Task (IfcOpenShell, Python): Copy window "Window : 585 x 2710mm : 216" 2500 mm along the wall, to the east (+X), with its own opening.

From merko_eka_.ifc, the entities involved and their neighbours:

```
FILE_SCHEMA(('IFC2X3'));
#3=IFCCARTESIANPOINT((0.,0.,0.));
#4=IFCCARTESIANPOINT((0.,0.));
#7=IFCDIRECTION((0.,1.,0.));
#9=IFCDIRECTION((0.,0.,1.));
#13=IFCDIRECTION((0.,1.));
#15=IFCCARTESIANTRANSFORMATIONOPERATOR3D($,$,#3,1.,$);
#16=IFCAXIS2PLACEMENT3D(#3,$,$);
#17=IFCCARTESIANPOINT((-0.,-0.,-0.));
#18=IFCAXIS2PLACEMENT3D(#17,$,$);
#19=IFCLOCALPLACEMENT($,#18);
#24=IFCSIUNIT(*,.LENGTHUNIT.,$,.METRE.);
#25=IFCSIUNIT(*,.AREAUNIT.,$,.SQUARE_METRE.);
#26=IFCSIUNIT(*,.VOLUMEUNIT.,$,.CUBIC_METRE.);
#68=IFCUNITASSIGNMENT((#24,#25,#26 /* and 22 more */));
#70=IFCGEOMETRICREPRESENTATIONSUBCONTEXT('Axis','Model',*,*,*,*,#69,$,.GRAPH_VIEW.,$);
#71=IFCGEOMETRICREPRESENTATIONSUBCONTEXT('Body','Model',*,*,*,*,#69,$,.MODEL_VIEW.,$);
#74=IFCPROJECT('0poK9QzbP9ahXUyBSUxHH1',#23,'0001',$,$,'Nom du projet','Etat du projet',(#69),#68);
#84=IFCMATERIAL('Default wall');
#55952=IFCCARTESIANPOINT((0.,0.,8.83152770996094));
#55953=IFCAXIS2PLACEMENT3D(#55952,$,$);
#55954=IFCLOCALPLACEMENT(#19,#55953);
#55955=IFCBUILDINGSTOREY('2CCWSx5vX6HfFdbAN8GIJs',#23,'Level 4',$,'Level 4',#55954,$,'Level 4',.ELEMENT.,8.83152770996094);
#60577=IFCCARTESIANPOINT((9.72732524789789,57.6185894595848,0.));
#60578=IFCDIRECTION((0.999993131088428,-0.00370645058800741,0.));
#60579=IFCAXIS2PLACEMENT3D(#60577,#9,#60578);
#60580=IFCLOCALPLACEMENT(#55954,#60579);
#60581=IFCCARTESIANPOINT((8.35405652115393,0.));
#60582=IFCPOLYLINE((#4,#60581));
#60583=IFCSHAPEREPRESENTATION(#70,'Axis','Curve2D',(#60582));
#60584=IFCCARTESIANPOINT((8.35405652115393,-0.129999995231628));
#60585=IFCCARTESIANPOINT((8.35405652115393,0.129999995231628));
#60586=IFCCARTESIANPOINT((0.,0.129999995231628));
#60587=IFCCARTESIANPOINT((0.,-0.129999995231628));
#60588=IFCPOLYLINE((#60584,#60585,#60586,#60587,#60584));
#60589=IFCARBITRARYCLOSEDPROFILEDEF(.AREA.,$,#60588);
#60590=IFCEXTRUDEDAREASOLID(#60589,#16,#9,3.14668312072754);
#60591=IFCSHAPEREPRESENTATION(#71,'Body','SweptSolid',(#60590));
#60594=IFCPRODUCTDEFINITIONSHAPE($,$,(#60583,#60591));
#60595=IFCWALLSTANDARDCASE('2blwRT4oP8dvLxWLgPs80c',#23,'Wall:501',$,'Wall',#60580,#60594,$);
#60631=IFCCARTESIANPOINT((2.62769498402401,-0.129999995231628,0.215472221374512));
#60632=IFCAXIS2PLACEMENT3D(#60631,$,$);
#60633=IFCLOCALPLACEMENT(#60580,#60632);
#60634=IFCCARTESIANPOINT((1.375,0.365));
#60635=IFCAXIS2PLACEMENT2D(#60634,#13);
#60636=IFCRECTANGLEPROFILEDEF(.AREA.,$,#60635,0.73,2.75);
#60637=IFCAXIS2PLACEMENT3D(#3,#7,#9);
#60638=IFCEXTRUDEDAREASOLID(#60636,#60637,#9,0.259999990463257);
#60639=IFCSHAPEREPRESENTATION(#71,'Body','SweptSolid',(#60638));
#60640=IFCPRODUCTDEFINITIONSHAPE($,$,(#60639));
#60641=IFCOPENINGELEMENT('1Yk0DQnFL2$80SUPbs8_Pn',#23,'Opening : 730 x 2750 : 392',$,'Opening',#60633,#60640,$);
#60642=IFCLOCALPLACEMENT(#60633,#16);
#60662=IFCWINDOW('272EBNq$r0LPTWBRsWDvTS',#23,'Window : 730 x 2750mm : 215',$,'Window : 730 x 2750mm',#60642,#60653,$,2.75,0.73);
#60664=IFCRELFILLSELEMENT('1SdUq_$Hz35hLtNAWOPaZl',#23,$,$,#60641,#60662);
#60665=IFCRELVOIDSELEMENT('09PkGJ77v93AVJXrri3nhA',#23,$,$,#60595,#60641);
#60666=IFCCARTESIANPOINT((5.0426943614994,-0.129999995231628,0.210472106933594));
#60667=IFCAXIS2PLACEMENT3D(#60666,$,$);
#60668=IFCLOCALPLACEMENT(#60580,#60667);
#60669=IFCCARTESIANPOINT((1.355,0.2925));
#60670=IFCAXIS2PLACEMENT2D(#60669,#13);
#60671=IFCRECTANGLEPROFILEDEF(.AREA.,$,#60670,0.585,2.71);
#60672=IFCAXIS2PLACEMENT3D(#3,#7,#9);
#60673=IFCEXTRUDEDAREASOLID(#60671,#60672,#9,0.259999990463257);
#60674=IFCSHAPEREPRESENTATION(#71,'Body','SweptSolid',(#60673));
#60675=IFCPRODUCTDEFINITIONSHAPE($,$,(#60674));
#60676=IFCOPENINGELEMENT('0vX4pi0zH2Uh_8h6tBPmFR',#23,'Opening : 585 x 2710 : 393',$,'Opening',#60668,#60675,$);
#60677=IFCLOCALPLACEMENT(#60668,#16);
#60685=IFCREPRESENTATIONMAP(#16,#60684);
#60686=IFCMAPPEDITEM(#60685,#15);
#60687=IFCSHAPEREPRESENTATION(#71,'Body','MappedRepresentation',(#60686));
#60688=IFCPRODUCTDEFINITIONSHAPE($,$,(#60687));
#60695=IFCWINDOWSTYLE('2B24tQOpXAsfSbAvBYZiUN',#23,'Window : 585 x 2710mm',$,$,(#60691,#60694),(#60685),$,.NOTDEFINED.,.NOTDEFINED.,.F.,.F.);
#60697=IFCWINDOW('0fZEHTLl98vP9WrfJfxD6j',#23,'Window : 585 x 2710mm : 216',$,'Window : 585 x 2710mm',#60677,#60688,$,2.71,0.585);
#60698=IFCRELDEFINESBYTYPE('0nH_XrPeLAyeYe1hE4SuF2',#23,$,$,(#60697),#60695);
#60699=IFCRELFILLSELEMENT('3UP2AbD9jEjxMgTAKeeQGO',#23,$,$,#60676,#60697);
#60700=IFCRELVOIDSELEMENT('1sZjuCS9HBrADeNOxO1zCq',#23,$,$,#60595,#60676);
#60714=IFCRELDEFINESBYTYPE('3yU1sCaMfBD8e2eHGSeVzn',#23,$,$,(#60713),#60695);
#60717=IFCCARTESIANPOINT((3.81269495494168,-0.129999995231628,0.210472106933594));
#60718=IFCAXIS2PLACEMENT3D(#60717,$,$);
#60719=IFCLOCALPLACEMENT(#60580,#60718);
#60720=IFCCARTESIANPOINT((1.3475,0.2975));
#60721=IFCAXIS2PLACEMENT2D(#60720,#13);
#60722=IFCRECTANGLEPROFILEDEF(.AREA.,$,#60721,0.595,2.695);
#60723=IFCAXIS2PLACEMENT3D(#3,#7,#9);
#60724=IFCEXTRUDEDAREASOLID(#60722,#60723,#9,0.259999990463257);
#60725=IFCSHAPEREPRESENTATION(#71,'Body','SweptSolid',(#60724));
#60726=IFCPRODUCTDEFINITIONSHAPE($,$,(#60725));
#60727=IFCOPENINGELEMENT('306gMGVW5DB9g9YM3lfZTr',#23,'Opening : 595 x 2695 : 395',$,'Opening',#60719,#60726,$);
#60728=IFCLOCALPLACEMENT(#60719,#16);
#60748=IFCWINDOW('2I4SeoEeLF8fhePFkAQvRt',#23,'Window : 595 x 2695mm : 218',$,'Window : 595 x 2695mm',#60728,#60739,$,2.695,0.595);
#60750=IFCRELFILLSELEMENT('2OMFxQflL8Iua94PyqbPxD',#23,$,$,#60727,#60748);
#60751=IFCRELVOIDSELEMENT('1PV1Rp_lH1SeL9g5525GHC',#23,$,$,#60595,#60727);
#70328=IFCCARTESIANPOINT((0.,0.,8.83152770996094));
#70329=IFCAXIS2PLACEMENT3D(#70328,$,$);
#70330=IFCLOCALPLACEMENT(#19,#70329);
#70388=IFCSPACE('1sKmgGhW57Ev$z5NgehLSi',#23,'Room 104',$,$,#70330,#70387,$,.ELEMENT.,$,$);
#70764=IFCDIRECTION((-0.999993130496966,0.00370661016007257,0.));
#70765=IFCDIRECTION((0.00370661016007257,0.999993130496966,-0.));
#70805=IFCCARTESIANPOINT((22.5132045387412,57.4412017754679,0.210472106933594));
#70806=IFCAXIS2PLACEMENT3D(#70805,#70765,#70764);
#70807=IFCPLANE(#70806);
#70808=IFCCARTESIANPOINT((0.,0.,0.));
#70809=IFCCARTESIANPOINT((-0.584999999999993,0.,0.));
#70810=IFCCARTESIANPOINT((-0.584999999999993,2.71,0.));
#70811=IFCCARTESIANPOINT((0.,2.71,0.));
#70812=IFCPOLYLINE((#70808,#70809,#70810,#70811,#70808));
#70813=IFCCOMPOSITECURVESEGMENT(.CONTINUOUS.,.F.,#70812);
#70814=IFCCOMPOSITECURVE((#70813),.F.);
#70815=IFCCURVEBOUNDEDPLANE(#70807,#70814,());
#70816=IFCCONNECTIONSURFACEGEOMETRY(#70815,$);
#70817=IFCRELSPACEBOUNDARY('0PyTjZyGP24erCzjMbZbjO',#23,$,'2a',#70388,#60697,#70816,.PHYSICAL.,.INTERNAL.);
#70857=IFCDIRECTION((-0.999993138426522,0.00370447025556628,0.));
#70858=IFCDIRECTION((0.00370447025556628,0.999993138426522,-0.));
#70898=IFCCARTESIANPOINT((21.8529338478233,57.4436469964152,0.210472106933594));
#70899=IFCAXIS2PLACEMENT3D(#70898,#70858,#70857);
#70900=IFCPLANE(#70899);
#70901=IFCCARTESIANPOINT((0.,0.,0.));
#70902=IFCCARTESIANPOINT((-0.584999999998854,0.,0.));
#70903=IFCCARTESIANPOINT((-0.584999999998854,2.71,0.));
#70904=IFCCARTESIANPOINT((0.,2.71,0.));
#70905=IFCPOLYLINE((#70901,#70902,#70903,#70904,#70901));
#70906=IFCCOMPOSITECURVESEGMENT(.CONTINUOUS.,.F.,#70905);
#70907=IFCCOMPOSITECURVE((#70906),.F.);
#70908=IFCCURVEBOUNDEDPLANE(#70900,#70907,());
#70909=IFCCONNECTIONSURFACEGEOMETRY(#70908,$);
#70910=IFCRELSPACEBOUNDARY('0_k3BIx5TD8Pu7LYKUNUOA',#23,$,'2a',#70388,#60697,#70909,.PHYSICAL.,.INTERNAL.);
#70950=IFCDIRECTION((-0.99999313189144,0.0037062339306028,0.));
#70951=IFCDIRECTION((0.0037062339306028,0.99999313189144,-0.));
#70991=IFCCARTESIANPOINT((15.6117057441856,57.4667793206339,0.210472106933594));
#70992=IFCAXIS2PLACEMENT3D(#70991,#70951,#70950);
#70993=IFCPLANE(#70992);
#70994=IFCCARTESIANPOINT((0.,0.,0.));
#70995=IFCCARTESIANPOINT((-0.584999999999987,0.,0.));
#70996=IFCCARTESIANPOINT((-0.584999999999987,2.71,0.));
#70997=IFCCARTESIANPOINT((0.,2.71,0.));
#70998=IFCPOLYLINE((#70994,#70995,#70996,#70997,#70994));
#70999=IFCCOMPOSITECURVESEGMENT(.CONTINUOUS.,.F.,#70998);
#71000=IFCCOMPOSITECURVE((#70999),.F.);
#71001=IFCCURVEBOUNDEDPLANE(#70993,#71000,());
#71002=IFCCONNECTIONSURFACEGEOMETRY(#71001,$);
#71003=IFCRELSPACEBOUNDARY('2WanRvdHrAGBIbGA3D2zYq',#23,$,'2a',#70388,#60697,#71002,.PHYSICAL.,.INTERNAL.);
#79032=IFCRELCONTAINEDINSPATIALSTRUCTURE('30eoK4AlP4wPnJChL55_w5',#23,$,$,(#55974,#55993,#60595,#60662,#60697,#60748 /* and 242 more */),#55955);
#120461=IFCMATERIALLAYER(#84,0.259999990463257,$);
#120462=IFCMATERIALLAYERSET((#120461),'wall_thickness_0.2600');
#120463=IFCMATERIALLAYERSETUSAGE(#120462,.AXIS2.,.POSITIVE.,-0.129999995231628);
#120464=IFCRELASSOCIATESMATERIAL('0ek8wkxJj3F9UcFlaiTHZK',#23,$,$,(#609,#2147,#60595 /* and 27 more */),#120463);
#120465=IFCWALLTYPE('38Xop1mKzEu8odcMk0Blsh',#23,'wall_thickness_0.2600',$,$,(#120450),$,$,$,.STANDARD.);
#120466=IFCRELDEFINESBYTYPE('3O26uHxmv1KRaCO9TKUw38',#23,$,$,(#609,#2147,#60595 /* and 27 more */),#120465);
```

```python
import numpy as np
import ifcopenshell
import ifcopenshell.api.feature
import ifcopenshell.api.geometry
import ifcopenshell.api.root
import ifcopenshell.geom
import ifcopenshell.util.element
import ifcopenshell.util.placement
import ifcopenshell.util.shape

model = ifcopenshell.open("merko_eka_.ifc")
settings = ifcopenshell.geom.settings()


def volume(element):
    """Net volume in cubic metres, openings subtracted."""
    shape = ifcopenshell.geom.create_shape(settings, element)
    return ifcopenshell.util.shape.get_volume(shape.geometry)


window = model.by_guid("0fZEHTLl98vP9WrfJfxD6j")
opening = window.FillsVoids[0].RelatingOpeningElement
wall = opening.VoidsElements[0].RelatingBuildingElement
before = volume(wall)
shift = ifcopenshell.util.placement.get_local_placement(wall.ObjectPlacement)[:3, 0] * 2.5

# copy_class copies the void relationship, type, container and properties, but no geometry.
new_opening = ifcopenshell.api.root.copy_class(model, product=opening)
new_opening.Representation = ifcopenshell.util.element.copy_deep(
    model, opening.Representation, exclude=["IfcGeometricRepresentationContext", "IfcRepresentationMap"]
)
new_opening.Name = "Opening : 585 x 2710"
new_window = ifcopenshell.api.root.copy_class(model, product=window)
new_window.Representation = ifcopenshell.util.element.copy_deep(
    model, window.Representation, exclude=["IfcGeometricRepresentationContext", "IfcRepresentationMap"]
)
new_window.Name = "Window : 585 x 2710mm"
fills = ifcopenshell.api.feature.add_filling(model, opening=new_opening, element=new_window)
fills.OwnerHistory = new_window.OwnerHistory  # required in IFC2X3

for old, new in ((opening, new_opening), (window, new_window)):
    matrix = ifcopenshell.util.placement.get_local_placement(old.ObjectPlacement)
    matrix[:3, 3] += shift
    ifcopenshell.api.geometry.edit_object_placement(model, product=new, matrix=matrix, is_si=False)

# The copied space boundaries still share their surfaces with the original.
for rel in new_window.ProvidesBoundaries:
    if rel.ConnectionGeometry:
        rel.ConnectionGeometry = ifcopenshell.util.element.copy_deep(model, rel.ConnectionGeometry)

# Space boundary surfaces are stored in each space's coordinates; move them too.
for rel in new_window.ProvidesBoundaries:
    if not rel.ConnectionGeometry:
        continue
    surface = rel.ConnectionGeometry.SurfaceOnRelatingElement.BasisSurface
    space_matrix = ifcopenshell.util.placement.get_local_placement(rel.RelatingSpace.ObjectPlacement)
    point = np.array(surface.Position.Location.Coordinates) + space_matrix[:3, :3].T @ shift
    surface.Position = model.createIfcAxis2Placement3D(
        model.createIfcCartesianPoint(point.tolist()), surface.Position.Axis, surface.Position.RefDirection
    )

after = volume(wall)

print(f"wall volume {before:.3f} -> {after:.3f} m3")

model.write("merko_eka__edited.ifc")
```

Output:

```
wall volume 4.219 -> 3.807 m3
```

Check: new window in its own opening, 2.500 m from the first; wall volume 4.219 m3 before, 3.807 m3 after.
